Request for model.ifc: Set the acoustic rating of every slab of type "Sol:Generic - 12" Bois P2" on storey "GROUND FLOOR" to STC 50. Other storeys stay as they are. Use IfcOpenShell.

First a look at what the model holds.

```python
import ifcopenshell
import ifcopenshell.util.element

model = ifcopenshell.open("model.ifc")
print(model.schema)
storey = next(s for s in model.by_type("IfcBuildingStorey") if s.Name == "GROUND FLOOR")
slabs = [e for e in ifcopenshell.util.element.get_decomposition(storey) if e.is_a("IfcSlab")]
seen = {}
for e in slabs:
    element_type = ifcopenshell.util.element.get_type(e)
    key = (element_type.Name if element_type != e and element_type else None, ifcopenshell.util.element.get_pset(e, "Pset_SlabCommon", "AcousticRating"))
    seen[key] = seen.get(key, 0) + 1
for (name, value), count in sorted(seen.items(), key=str):
    print(count, "x", name, "|", value)
```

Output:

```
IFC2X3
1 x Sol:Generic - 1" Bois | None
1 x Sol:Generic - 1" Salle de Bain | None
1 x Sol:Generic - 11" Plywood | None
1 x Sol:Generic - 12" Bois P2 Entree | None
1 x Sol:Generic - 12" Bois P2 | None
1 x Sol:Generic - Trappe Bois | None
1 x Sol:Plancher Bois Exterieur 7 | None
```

```python
import ifcopenshell
import ifcopenshell.api.pset
import ifcopenshell.util.element

model = ifcopenshell.open("model.ifc")

storey = next(s for s in model.by_type("IfcBuildingStorey") if s.Name == "GROUND FLOOR")
slabs = [e for e in ifcopenshell.util.element.get_decomposition(storey) if e.is_a("IfcSlab")]

count = 0
for e in slabs:
    element_type = ifcopenshell.util.element.get_type(e)
    if element_type in (None, e) or element_type.Name != 'Sol:Generic - 12" Bois P2':
        continue
    # add_pset returns the element's existing set when there is one.
    pset = ifcopenshell.api.pset.add_pset(model, product=e, name="Pset_SlabCommon")
    ifcopenshell.api.pset.edit_pset(model, pset=pset, properties={"AcousticRating": "STC 50"})
    count += 1

print(count, "slabs updated")

model.write("model-out.ifc")
```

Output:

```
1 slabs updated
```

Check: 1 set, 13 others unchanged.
